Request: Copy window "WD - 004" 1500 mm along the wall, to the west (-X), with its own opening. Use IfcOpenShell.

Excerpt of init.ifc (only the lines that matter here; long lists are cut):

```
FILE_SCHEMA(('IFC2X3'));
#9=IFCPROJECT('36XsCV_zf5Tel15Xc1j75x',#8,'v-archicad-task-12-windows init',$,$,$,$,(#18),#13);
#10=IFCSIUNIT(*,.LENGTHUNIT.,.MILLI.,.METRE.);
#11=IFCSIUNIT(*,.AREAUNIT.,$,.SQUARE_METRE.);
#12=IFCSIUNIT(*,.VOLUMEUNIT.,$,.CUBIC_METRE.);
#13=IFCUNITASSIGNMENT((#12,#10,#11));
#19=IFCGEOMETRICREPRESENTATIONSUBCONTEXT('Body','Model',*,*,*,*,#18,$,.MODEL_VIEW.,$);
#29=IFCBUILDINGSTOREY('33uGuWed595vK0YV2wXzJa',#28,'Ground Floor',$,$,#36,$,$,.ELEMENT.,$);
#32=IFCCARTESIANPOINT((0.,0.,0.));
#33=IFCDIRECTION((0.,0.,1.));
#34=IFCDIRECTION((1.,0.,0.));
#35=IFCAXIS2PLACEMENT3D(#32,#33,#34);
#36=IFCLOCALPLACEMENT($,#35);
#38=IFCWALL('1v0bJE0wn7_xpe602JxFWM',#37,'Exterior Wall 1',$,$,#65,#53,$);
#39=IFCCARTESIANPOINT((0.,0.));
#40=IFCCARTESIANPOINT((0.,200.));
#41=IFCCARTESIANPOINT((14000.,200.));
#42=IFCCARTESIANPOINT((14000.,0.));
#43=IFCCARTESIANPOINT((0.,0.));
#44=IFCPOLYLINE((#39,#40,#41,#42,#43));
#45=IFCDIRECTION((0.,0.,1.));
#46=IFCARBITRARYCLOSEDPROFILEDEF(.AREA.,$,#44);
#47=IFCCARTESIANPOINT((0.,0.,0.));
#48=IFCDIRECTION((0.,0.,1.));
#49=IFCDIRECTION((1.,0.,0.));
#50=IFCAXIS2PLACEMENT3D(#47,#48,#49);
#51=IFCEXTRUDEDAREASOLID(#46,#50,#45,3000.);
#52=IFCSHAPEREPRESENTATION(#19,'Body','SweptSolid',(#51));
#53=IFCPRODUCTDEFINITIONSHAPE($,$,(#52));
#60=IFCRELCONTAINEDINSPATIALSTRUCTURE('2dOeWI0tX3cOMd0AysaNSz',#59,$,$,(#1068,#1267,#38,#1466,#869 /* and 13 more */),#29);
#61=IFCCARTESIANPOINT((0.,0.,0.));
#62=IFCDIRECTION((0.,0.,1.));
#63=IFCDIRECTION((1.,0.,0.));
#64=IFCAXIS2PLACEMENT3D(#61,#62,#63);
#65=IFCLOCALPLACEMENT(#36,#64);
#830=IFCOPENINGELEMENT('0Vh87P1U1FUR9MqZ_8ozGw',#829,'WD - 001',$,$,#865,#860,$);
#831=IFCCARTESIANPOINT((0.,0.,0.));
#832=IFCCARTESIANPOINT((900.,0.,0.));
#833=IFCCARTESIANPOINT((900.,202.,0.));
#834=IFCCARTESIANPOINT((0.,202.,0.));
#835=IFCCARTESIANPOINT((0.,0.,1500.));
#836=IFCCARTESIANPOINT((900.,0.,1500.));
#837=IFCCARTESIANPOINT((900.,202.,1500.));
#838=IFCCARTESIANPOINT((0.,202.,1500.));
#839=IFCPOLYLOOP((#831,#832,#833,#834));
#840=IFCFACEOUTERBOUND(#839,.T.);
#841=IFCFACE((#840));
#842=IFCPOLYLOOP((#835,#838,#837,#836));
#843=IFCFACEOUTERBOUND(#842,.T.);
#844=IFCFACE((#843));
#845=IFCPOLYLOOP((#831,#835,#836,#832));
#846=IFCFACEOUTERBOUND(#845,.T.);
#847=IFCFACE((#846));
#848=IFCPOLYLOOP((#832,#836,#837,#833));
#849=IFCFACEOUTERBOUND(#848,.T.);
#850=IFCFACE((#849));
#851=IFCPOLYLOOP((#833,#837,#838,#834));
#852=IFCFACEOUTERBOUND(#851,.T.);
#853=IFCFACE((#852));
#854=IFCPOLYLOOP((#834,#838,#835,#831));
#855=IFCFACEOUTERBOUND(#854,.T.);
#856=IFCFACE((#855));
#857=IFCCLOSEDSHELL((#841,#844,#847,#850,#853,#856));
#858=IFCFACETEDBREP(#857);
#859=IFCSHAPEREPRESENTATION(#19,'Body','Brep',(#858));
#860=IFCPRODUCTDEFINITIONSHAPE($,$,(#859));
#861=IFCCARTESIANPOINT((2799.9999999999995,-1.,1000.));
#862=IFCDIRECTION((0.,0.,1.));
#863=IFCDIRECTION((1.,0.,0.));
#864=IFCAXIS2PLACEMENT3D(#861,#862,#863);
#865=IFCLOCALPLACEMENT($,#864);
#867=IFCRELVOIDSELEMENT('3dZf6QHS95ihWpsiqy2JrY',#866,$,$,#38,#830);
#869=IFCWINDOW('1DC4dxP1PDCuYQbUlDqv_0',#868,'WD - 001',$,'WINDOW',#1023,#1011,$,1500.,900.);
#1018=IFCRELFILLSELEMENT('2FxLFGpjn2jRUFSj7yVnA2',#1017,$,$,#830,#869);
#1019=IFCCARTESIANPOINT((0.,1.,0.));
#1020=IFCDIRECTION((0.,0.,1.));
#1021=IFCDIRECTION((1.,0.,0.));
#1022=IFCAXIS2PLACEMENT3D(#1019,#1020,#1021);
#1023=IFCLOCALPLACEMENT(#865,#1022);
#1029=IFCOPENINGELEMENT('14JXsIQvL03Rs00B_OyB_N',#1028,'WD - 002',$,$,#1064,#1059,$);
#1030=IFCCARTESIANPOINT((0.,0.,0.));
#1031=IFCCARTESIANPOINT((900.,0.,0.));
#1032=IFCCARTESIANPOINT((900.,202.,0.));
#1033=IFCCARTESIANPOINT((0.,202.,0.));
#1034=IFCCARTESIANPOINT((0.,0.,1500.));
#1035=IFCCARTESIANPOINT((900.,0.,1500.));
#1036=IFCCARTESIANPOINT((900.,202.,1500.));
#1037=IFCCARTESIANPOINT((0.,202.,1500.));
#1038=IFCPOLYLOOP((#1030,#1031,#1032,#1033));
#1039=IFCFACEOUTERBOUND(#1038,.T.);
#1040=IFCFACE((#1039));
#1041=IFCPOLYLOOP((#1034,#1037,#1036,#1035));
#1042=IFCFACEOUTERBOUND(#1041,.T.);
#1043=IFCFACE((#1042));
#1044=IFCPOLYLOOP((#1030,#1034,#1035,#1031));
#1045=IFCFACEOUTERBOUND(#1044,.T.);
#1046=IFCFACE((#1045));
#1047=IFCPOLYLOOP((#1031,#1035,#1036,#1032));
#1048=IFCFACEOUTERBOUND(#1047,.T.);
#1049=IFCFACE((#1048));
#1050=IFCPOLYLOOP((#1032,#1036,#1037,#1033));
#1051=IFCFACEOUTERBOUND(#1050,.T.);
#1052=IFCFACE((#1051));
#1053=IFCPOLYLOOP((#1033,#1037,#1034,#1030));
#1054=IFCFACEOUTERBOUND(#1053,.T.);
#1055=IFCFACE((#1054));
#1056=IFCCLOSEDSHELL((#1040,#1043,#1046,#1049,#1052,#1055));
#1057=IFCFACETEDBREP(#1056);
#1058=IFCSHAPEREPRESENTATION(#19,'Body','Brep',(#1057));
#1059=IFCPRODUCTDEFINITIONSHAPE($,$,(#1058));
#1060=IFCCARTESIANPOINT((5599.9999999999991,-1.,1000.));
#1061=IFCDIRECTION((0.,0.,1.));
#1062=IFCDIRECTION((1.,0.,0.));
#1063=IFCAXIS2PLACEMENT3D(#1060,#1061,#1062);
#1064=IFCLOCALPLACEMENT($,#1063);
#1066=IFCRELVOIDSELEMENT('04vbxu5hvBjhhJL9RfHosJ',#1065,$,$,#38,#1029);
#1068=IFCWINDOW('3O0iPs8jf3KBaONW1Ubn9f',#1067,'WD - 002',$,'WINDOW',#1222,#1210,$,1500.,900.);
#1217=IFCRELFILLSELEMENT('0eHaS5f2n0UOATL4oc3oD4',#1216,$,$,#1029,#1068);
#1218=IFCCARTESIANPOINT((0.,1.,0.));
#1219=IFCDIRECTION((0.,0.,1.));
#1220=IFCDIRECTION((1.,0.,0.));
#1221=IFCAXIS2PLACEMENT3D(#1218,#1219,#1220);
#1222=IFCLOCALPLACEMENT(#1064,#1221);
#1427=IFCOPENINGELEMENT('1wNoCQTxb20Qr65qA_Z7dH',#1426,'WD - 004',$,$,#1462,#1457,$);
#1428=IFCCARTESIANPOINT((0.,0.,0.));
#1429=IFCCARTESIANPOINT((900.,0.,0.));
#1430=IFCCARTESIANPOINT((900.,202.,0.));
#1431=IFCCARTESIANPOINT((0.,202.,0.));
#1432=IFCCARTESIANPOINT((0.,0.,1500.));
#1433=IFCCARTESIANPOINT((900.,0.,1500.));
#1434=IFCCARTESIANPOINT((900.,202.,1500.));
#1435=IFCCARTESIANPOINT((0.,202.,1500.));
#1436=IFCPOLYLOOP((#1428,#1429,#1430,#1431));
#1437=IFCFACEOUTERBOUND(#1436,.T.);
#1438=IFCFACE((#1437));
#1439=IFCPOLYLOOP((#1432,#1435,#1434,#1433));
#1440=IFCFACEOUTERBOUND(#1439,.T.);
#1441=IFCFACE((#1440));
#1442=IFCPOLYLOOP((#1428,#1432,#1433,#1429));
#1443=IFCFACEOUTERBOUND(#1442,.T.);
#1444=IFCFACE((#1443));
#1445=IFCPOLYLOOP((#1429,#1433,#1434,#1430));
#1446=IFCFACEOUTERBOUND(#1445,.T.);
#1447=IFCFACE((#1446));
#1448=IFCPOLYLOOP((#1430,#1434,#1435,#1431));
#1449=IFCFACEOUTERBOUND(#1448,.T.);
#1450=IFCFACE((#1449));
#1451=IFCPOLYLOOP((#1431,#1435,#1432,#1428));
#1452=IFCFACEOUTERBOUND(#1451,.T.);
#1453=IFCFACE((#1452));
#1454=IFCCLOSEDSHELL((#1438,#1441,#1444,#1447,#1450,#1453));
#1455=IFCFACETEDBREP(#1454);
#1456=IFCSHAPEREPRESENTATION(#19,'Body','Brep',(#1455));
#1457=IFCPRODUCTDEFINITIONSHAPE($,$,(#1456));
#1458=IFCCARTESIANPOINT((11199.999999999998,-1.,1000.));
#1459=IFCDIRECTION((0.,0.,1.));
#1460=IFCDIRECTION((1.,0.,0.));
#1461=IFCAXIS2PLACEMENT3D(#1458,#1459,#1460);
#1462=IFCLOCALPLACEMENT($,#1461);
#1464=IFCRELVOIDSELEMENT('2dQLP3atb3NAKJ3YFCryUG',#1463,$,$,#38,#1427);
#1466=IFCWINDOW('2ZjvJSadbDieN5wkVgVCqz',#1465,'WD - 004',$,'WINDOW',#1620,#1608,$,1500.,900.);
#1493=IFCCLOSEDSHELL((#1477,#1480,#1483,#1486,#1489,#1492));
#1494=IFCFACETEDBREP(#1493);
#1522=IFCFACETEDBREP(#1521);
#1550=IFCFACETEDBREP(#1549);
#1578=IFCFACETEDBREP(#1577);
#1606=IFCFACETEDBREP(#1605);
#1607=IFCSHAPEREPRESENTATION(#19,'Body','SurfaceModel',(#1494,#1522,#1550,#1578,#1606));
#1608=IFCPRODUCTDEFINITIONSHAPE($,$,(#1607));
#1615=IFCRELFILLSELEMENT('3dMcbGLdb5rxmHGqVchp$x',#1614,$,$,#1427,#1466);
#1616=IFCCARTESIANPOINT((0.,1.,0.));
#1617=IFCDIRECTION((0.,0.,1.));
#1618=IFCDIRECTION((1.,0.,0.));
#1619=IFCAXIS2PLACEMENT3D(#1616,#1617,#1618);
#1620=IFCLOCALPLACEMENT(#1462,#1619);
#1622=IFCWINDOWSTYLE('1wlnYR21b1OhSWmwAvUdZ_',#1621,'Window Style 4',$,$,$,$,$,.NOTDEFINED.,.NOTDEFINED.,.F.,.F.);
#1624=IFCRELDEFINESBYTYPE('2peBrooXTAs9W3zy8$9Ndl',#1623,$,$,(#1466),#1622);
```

```python
import ifcopenshell
import ifcopenshell.api.feature
import ifcopenshell.api.geometry
import ifcopenshell.api.root
import ifcopenshell.geom
import ifcopenshell.util.element
import ifcopenshell.util.placement
import ifcopenshell.util.shape

model = ifcopenshell.open("init.ifc")
settings = ifcopenshell.geom.settings()


def volume(element):
    """Net volume in cubic metres, openings subtracted."""
    shape = ifcopenshell.geom.create_shape(settings, element)
    return ifcopenshell.util.shape.get_volume(shape.geometry)


window = model.by_guid("2ZjvJSadbDieN5wkVgVCqz")
opening = window.FillsVoids[0].RelatingOpeningElement
wall = opening.VoidsElements[0].RelatingBuildingElement
before = volume(wall)
shift = ifcopenshell.util.placement.get_local_placement(wall.ObjectPlacement)[:3, 0] * -1500.0

# copy_class copies the void relationship, type, container and properties, but no geometry.
new_opening = ifcopenshell.api.root.copy_class(model, product=opening)
new_opening.Representation = ifcopenshell.util.element.copy_deep(
    model, opening.Representation, exclude=["IfcGeometricRepresentationContext", "IfcRepresentationMap"]
)
new_window = ifcopenshell.api.root.copy_class(model, product=window)
new_window.Representation = ifcopenshell.util.element.copy_deep(
    model, window.Representation, exclude=["IfcGeometricRepresentationContext", "IfcRepresentationMap"]
)
fills = ifcopenshell.api.feature.add_filling(model, opening=new_opening, element=new_window)
fills.OwnerHistory = new_window.OwnerHistory  # required in IFC2X3

for old, new in ((opening, new_opening), (window, new_window)):
    matrix = ifcopenshell.util.placement.get_local_placement(old.ObjectPlacement)
    matrix[:3, 3] += shift
    ifcopenshell.api.geometry.edit_object_placement(model, product=new, matrix=matrix, is_si=False)

after = volume(wall)

print(f"wall volume {before:.3f} -> {after:.3f} m3")

model.write("init_v2.ifc")
```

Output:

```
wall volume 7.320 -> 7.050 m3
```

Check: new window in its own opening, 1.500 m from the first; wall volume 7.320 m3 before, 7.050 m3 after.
